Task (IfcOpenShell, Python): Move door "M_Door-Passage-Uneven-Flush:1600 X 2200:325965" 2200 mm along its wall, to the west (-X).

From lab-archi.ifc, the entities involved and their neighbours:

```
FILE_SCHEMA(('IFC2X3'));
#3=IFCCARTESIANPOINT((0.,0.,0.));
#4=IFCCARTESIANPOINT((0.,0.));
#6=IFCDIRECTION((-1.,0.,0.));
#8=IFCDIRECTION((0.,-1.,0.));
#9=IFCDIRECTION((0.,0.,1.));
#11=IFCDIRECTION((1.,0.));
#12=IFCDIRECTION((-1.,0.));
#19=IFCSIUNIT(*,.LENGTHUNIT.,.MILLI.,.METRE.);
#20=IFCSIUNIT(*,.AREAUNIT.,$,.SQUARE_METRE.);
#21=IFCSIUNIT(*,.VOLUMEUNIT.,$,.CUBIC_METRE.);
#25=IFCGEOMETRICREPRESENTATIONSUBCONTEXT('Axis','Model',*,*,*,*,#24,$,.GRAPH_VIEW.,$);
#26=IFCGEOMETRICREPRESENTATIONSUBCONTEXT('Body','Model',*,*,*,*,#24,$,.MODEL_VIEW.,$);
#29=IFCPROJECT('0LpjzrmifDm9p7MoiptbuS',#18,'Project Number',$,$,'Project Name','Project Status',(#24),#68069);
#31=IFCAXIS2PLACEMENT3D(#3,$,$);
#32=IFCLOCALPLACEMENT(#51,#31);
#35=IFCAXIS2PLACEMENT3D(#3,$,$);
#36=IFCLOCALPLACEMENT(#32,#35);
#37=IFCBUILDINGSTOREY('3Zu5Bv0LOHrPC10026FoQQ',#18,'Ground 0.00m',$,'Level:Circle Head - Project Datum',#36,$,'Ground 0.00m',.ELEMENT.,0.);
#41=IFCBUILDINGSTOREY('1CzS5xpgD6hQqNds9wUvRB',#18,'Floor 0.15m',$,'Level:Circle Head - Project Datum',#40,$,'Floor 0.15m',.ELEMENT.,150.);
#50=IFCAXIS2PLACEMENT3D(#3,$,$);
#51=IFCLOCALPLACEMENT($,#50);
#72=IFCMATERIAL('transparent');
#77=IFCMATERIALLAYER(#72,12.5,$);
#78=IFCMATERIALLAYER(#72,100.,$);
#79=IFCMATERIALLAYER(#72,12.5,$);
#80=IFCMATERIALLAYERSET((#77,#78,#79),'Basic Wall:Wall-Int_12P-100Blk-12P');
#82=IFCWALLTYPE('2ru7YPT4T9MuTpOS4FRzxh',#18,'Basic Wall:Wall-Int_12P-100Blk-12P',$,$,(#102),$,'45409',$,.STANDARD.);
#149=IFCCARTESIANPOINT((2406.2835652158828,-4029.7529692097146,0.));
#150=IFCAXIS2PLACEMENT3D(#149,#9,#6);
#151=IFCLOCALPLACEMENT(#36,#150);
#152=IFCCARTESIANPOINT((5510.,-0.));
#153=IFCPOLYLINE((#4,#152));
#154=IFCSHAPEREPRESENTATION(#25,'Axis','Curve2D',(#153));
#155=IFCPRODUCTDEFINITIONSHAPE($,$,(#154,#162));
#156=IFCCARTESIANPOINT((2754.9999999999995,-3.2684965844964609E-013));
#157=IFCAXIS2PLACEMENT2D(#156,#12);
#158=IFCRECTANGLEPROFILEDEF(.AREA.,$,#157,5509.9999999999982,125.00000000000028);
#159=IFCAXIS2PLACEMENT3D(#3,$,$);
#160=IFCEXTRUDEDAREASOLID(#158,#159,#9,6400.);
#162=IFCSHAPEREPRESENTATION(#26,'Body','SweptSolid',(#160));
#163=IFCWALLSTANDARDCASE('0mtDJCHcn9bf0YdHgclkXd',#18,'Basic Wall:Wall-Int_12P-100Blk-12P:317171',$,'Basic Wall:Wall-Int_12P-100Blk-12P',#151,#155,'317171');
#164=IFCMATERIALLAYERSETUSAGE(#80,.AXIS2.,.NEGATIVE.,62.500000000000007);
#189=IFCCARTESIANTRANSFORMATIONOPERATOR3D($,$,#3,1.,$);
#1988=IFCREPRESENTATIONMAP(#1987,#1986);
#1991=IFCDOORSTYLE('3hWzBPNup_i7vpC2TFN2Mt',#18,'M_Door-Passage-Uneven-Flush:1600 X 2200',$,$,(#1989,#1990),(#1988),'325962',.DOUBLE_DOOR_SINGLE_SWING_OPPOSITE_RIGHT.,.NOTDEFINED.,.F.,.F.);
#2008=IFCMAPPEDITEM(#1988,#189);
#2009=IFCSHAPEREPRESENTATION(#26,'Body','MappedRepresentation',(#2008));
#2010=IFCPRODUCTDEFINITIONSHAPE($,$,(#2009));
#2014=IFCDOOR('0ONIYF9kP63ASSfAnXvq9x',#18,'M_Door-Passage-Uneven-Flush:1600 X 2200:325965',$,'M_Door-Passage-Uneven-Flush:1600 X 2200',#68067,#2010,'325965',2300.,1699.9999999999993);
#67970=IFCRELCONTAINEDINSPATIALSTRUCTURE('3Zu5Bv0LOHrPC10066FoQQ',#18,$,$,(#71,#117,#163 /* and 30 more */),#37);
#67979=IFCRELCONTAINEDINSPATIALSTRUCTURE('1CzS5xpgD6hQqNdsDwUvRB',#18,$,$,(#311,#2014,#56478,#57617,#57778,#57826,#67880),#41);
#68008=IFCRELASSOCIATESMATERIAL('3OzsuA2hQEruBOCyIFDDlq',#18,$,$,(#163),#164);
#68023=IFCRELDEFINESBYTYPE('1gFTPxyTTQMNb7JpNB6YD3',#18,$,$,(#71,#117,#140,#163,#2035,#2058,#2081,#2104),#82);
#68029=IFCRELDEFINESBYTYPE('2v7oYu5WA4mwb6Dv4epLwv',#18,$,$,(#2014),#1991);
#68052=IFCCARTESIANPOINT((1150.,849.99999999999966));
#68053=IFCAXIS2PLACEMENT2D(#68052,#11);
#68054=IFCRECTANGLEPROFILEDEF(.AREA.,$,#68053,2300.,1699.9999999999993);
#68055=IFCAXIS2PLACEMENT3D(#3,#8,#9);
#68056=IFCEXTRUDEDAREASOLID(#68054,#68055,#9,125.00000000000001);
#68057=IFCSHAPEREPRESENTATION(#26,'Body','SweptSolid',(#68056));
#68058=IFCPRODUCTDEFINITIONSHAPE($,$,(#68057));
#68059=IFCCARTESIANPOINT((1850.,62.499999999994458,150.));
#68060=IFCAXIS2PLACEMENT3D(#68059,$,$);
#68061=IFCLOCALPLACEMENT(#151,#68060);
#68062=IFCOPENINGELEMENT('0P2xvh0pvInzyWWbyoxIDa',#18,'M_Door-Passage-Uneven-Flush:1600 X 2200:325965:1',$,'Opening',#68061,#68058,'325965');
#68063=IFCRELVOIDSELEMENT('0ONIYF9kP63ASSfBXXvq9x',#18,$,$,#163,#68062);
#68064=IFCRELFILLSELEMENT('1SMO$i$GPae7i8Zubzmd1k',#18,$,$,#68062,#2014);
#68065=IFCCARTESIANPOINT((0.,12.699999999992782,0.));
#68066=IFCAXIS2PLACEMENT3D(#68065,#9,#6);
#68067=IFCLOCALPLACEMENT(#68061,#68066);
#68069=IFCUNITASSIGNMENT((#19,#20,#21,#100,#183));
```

```python
import ifcopenshell
import ifcopenshell.api.geometry
import ifcopenshell.util.placement

model = ifcopenshell.open("lab-archi.ifc")

door = model.by_id(2014)
opening = door.FillsVoids[0].RelatingOpeningElement
wall = opening.VoidsElements[0].RelatingBuildingElement

wall_matrix = ifcopenshell.util.placement.get_local_placement(wall.ObjectPlacement)
shift = wall_matrix[:3, 0] * 2200.0
before = ifcopenshell.util.placement.get_local_placement(door.ObjectPlacement)[:3, 3].copy()

# The door is placed relative to its opening, so it follows when the opening moves.
matrix = ifcopenshell.util.placement.get_local_placement(opening.ObjectPlacement)
matrix[:3, 3] += shift
ifcopenshell.api.geometry.edit_object_placement(
    model, product=opening, matrix=matrix, is_si=False, should_transform_children=True
)

after = ifcopenshell.util.placement.get_local_placement(door.ObjectPlacement)[:3, 3]
print("door moved by", (after - before).round(3) + 0.0)

model.write("lab-archi-out.ifc")
```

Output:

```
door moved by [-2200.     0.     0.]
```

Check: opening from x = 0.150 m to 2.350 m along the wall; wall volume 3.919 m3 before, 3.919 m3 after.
